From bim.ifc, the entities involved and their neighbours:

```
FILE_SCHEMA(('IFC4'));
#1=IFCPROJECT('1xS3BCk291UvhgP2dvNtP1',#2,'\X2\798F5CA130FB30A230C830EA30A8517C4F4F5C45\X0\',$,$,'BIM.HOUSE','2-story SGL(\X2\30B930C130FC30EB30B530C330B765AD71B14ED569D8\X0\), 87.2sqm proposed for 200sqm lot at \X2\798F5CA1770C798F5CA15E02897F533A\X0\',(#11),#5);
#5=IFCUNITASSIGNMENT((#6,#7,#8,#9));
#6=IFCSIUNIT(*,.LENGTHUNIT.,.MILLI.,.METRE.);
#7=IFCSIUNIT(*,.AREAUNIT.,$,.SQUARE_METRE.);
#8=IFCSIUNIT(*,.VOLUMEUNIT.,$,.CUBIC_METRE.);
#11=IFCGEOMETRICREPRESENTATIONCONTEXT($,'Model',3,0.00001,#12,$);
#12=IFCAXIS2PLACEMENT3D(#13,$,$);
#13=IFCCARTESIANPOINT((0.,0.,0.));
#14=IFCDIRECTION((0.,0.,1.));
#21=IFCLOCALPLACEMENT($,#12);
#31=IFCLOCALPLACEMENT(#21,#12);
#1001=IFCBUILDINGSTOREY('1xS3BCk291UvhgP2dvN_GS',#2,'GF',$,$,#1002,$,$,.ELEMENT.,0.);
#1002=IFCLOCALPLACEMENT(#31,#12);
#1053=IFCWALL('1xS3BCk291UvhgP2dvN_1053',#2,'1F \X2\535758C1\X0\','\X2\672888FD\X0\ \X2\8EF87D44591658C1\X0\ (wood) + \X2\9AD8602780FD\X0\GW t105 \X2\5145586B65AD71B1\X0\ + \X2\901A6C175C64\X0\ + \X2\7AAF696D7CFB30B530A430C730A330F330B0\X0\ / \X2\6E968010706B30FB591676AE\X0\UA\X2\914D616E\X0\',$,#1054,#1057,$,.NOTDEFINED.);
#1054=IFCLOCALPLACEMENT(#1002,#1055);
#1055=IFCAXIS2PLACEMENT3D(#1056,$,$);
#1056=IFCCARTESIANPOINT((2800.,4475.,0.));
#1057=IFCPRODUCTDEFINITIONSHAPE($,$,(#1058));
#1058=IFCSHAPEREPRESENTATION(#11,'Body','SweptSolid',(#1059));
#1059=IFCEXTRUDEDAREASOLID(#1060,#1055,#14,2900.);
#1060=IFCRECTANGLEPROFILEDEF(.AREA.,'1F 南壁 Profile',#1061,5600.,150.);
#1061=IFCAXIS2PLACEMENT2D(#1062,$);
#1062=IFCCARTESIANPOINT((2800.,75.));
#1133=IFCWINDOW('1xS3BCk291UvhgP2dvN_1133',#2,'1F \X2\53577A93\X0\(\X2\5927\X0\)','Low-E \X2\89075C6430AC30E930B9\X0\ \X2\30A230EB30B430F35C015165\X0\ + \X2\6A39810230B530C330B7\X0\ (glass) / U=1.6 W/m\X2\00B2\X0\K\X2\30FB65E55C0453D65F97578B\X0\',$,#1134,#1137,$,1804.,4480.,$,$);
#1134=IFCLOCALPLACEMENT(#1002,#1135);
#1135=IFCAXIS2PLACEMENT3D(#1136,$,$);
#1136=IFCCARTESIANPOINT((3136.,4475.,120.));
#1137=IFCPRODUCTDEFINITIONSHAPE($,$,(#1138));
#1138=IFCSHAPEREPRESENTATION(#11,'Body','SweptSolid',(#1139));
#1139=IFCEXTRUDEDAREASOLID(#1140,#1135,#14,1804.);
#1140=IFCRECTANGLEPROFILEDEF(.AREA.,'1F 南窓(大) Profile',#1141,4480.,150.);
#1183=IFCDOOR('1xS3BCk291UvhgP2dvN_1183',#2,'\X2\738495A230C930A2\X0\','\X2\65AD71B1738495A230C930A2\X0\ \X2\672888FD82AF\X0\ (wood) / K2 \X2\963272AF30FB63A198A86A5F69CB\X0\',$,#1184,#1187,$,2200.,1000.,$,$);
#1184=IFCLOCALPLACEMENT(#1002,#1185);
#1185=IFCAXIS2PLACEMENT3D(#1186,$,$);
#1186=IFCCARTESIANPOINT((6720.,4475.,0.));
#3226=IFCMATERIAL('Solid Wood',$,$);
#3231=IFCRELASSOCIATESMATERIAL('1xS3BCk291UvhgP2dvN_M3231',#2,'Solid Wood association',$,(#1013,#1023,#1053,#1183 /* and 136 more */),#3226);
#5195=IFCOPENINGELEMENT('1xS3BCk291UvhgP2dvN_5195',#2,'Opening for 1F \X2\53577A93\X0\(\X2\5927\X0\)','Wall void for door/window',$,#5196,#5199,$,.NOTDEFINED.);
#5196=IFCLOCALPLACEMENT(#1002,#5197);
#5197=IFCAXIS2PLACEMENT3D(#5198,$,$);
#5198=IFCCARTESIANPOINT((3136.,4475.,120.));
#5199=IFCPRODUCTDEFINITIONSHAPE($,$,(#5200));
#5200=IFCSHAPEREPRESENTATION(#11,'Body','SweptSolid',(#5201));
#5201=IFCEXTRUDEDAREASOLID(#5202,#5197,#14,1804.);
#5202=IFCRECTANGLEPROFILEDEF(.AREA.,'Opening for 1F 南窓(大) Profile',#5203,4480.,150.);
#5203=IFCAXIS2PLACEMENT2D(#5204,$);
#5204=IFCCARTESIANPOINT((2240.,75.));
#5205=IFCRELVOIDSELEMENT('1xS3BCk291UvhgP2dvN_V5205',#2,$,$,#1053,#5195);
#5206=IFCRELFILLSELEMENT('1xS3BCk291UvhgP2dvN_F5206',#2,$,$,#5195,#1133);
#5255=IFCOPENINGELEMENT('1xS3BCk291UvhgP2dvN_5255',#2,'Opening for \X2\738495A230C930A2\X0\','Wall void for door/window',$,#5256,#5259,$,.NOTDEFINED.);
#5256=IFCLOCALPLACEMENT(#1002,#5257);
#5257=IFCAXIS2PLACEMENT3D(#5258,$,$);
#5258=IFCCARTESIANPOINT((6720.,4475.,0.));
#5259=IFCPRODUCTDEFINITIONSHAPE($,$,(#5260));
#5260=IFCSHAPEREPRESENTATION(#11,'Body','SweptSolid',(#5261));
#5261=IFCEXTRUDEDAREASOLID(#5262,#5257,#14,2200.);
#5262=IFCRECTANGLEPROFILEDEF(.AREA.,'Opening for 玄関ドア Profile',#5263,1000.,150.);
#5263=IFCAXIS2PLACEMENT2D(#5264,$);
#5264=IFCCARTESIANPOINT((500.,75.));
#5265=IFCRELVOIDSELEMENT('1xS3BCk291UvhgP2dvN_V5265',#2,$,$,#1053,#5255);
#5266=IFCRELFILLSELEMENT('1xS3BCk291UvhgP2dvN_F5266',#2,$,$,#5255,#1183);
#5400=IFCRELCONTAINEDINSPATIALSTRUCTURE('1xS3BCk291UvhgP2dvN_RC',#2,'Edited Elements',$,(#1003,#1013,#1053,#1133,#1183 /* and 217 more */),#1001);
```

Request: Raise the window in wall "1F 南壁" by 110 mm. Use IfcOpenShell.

```python
import numpy as np
import ifcopenshell
import ifcopenshell.api.geometry
import ifcopenshell.util.placement
import ifcopenshell.util.unit

model = ifcopenshell.open("bim.ifc")
unit_scale = ifcopenshell.util.unit.calculate_unit_scale(model)

window = model.by_guid("1xS3BCk291UvhgP2dvN_1133")
opening = window.FillsVoids[0].RelatingOpeningElement
dz = 0.11 / unit_scale

shift = np.array([0.0, 0.0, dz])
# The window is not placed relative to its opening, so move both.
for product in (opening, window):
    matrix = ifcopenshell.util.placement.get_local_placement(product.ObjectPlacement)
    matrix[:3, 3] += shift
    ifcopenshell.api.geometry.edit_object_placement(model, product=product, matrix=matrix, is_si=False)

print(f"moved by {dz * unit_scale:+.3f} m")

model.write("bim-out.ifc")
```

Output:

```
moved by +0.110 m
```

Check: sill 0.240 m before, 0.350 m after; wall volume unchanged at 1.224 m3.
